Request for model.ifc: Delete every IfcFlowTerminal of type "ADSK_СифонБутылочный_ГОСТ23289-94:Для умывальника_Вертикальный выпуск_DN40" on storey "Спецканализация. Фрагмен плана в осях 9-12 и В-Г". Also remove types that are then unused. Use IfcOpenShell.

First a look at what the model holds.

```python
import ifcopenshell
import ifcopenshell.util.element

model = ifcopenshell.open("model.ifc")
print(model.schema)
storey = next(s for s in model.by_type("IfcBuildingStorey") if s.Name == "Спецканализация. Фрагмен плана в осях 9-12 и В-Г")
terminals = [e for e in ifcopenshell.util.element.get_decomposition(storey) if e.is_a("IfcFlowTerminal")]
seen = {}
for e in terminals:
    element_type = ifcopenshell.util.element.get_type(e)
    name = element_type.Name if element_type not in (None, e) else None
    seen[name] = seen.get(name, 0) + 1
for name, count in sorted(seen.items(), key=str):
    print(count, "x", name)
```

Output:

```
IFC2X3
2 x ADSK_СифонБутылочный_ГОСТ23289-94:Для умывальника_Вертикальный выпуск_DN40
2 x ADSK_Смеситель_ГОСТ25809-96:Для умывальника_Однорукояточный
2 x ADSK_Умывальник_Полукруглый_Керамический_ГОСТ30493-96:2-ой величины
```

```python
import ifcopenshell
import ifcopenshell.api.root
import ifcopenshell.util.element

model = ifcopenshell.open("model.ifc")

storey = next(s for s in model.by_type("IfcBuildingStorey") if s.Name == "Спецканализация. Фрагмен плана в осях 9-12 и В-Г")
terminals = [e for e in ifcopenshell.util.element.get_decomposition(storey) if e.is_a("IfcFlowTerminal")]
targets = [e for e in terminals if (t := ifcopenshell.util.element.get_type(e)) not in (None, e) and t.Name == "ADSK_СифонБутылочный_ГОСТ23289-94:Для умывальника_Вертикальный выпуск_DN40"]
types = {ifcopenshell.util.element.get_type(e) for e in targets} - {None, *targets}

for e in targets:
    ifcopenshell.api.root.remove_product(model, product=e)
print(len(targets), "removed")

unused = [t for t in types if not ifcopenshell.util.element.get_types(t)]
for t in unused:
    ifcopenshell.api.root.remove_product(model, product=t)
print(len(unused), "unused types removed")

model.write("model-out.ifc")
```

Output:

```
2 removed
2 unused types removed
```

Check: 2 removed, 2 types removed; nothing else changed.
